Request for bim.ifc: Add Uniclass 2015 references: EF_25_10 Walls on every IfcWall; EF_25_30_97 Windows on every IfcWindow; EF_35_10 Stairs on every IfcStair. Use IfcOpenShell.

First a look at what the model holds.

```python
import ifcopenshell

model = ifcopenshell.open("bim.ifc")
print(model.schema)
print("classifications:", [c.Name for c in model.by_type("IfcClassification")])
for ifc_class in ("IfcDoor", "IfcRoof", "IfcStair", "IfcWall", "IfcWindow"):
    print(ifc_class, len(model.by_type(ifc_class)))
```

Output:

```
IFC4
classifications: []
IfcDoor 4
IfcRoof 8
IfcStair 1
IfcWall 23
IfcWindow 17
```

```python
import ifcopenshell
import ifcopenshell.api.classification

model = ifcopenshell.open("bim.ifc")

system = ifcopenshell.api.classification.add_classification(model, classification="Uniclass 2015")

codes = {
    "IfcWall": ("EF_25_10", "Walls"),
    "IfcWindow": ("EF_25_30_97", "Windows"),
    "IfcStair": ("EF_35_10", "Stairs"),
}
for ifc_class, (code, name) in codes.items():
    products = model.by_type(ifc_class)
    ifcopenshell.api.classification.add_reference(
        model, products=products, classification=system, identification=code, name=name
    )
    print(code, len(products))

model.write("bim_v2.ifc")
```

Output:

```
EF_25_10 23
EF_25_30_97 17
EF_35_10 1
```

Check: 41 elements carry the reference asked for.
